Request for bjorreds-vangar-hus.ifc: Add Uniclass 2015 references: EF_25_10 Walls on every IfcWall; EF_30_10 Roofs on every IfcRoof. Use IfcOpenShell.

First a look at what the model holds.

```python
import ifcopenshell

model = ifcopenshell.open("bjorreds-vangar-hus.ifc")
print(model.schema)
print("classifications:", [c.Name for c in model.by_type("IfcClassification")])
for ifc_class in ("IfcDoor", "IfcRoof", "IfcStair", "IfcWall", "IfcWindow"):
    print(ifc_class, len(model.by_type(ifc_class)))
```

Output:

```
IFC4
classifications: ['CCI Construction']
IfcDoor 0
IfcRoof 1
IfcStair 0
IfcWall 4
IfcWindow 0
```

```python
import ifcopenshell
import ifcopenshell.api.classification

model = ifcopenshell.open("bjorreds-vangar-hus.ifc")

system = ifcopenshell.api.classification.add_classification(model, classification="Uniclass 2015")

codes = {
    "IfcWall": ("EF_25_10", "Walls"),
    "IfcRoof": ("EF_30_10", "Roofs"),
}
for ifc_class, (code, name) in codes.items():
    products = model.by_type(ifc_class)
    ifcopenshell.api.classification.add_reference(
        model, products=products, classification=system, identification=code, name=name
    )
    print(code, len(products))

model.write("bjorreds-vangar-hus_edited.ifc")
```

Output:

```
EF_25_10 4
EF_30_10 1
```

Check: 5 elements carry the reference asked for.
